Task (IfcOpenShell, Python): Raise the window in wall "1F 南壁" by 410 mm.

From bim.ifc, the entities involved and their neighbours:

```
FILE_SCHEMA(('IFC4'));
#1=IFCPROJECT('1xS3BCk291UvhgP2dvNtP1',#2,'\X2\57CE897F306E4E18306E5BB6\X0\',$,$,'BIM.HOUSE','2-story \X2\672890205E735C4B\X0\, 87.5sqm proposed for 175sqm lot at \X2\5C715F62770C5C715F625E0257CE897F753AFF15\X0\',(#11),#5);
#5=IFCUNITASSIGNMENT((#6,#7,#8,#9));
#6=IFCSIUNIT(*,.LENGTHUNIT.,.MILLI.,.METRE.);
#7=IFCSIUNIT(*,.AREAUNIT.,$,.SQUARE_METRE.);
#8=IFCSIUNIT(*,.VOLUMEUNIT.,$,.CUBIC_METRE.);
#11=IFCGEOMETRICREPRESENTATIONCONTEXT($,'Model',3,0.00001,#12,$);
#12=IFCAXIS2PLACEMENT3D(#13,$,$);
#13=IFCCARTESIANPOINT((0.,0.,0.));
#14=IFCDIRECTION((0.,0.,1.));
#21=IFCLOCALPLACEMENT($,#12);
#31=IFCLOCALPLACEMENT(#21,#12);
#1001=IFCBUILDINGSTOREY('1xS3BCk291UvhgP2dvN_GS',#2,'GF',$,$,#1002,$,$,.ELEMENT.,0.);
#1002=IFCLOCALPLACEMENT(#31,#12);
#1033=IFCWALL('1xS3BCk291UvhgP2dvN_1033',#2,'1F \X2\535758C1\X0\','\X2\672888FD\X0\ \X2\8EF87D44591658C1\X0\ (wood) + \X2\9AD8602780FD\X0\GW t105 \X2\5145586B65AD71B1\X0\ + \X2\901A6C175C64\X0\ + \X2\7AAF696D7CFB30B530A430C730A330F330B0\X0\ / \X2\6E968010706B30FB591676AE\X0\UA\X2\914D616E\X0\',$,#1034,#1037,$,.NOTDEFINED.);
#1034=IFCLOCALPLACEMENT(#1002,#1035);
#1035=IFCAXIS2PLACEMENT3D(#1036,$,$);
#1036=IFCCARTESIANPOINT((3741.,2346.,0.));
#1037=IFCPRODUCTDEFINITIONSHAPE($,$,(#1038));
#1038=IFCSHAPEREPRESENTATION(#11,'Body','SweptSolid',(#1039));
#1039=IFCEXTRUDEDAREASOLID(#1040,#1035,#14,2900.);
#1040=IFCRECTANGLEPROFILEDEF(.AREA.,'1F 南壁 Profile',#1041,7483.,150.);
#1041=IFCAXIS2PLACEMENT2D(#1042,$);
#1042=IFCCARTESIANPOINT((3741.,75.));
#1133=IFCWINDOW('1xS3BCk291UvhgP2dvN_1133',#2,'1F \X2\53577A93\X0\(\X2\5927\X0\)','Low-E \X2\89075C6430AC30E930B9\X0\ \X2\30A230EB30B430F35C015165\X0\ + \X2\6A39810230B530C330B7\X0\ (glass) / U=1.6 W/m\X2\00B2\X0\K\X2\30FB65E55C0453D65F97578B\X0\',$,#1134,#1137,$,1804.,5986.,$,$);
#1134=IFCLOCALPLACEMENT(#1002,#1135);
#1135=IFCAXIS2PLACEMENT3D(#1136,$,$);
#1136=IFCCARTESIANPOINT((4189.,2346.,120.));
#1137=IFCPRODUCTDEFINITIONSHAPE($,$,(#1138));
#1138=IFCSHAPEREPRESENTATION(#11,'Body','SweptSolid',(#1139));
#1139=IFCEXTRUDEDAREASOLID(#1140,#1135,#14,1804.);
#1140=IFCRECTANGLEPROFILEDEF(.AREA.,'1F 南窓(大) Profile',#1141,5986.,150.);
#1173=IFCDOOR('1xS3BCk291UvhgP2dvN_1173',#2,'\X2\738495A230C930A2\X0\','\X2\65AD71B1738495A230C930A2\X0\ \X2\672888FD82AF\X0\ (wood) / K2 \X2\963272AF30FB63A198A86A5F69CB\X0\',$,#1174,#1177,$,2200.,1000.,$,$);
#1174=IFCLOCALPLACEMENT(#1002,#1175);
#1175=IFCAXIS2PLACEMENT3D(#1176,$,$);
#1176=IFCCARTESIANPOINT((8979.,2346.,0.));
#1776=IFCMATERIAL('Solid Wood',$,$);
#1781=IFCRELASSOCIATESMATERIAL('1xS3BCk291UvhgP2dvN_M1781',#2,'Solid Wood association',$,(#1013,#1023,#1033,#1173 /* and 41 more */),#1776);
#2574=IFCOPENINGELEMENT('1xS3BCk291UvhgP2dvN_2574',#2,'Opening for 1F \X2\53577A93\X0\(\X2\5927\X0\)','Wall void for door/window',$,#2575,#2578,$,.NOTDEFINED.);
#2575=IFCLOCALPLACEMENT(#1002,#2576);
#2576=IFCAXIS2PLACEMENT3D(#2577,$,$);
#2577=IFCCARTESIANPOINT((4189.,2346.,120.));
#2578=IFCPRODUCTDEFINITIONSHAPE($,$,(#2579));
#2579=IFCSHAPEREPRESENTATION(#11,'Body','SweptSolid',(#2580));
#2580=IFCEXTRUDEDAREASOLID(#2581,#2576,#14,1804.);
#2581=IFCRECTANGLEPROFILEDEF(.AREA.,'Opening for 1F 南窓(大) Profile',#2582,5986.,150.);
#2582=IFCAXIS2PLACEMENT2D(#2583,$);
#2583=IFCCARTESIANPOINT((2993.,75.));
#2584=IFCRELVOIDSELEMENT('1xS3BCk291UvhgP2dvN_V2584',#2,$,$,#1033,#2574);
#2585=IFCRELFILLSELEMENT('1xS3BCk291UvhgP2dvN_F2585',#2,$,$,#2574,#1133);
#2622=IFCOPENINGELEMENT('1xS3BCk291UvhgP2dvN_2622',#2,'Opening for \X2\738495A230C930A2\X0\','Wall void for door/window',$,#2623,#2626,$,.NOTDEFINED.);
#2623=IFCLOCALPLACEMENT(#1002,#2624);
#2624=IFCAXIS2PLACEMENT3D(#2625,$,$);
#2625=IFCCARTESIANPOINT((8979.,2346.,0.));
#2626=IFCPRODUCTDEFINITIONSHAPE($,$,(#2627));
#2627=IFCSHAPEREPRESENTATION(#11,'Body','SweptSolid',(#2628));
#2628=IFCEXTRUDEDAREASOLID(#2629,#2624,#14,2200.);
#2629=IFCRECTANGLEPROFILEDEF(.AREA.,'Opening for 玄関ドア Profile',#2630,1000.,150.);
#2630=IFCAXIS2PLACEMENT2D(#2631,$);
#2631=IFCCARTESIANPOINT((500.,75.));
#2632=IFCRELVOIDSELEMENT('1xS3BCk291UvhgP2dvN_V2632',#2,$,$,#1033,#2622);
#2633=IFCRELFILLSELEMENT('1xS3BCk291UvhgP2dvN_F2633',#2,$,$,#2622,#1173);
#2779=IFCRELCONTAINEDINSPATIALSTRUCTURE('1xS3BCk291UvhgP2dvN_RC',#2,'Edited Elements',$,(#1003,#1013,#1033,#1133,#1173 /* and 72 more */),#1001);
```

```python
import numpy as np
import ifcopenshell
import ifcopenshell.api.geometry
import ifcopenshell.util.placement
import ifcopenshell.util.unit

model = ifcopenshell.open("bim.ifc")
unit_scale = ifcopenshell.util.unit.calculate_unit_scale(model)

window = model.by_guid("1xS3BCk291UvhgP2dvN_1133")
opening = window.FillsVoids[0].RelatingOpeningElement
dz = 0.41 / unit_scale

shift = np.array([0.0, 0.0, dz])
# The window is not placed relative to its opening, so move both.
for product in (opening, window):
    matrix = ifcopenshell.util.placement.get_local_placement(product.ObjectPlacement)
    matrix[:3, 3] += shift
    ifcopenshell.api.geometry.edit_object_placement(model, product=product, matrix=matrix, is_si=False)

print(f"moved by {dz * unit_scale:+.3f} m")

model.write("bim_edited.ifc")
```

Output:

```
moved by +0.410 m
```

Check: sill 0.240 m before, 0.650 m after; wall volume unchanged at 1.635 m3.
